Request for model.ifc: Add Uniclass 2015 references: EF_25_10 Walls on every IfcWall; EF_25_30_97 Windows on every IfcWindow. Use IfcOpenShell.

First a look at what the model holds.

```python
import ifcopenshell

model = ifcopenshell.open("model.ifc")
print(model.schema)
print("classifications:", [c.Name for c in model.by_type("IfcClassification")])
for ifc_class in ("IfcDoor", "IfcRoof", "IfcStair", "IfcWall", "IfcWindow"):
    print(ifc_class, len(model.by_type(ifc_class)))
```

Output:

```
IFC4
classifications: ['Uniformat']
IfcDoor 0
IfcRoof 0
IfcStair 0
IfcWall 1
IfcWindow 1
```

```python
import ifcopenshell
import ifcopenshell.api.classification

model = ifcopenshell.open("model.ifc")

system = ifcopenshell.api.classification.add_classification(model, classification="Uniclass 2015")

codes = {
    "IfcWall": ("EF_25_10", "Walls"),
    "IfcWindow": ("EF_25_30_97", "Windows"),
}
for ifc_class, (code, name) in codes.items():
    products = model.by_type(ifc_class)
    ifcopenshell.api.classification.add_reference(
        model, products=products, classification=system, identification=code, name=name
    )
    print(code, len(products))

model.write("model-out.ifc")
```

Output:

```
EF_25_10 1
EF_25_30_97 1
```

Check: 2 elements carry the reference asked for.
